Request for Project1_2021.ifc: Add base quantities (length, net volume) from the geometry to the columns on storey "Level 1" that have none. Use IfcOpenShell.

First a look at what the model holds.

```python
import ifcopenshell
import ifcopenshell.util.element
import ifcopenshell.util.unit

model = ifcopenshell.open("Project1_2021.ifc")
print(model.schema)
for unit_type in ("LENGTHUNIT", "AREAUNIT", "VOLUMEUNIT"):
    print(unit_type, ifcopenshell.util.unit.calculate_unit_scale(model, unit_type))
storey = next(s for s in model.by_type("IfcBuildingStorey") if s.Name == "Level 1")
columns = [e for e in ifcopenshell.util.element.get_decomposition(storey) if e.is_a("IfcColumn")]
for e in sorted(columns, key=lambda e: e.id()):
    print(e.id(), e.is_a(), e.Name, list(ifcopenshell.util.element.get_psets(e, qtos_only=True)), sep=" | ")
```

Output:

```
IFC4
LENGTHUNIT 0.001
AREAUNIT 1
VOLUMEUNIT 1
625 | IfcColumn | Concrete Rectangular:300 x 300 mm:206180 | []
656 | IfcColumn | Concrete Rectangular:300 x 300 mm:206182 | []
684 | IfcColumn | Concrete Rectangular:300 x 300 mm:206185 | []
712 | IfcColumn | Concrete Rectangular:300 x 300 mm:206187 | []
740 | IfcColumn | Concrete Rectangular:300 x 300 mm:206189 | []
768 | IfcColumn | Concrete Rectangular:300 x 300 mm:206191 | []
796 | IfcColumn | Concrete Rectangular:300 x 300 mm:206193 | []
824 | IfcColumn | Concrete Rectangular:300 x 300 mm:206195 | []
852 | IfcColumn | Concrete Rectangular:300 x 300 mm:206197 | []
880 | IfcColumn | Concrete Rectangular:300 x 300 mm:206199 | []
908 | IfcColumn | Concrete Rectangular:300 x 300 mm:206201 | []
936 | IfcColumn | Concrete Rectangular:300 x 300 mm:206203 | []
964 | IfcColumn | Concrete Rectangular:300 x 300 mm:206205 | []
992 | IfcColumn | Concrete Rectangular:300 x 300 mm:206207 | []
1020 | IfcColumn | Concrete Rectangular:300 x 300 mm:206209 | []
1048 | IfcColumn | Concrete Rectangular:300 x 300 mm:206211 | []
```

```python
import ifcopenshell
import ifcopenshell.api.pset
import ifcopenshell.geom
import ifcopenshell.util.element
import ifcopenshell.util.shape
import ifcopenshell.util.unit

model = ifcopenshell.open("Project1_2021.ifc")
unit_scale = ifcopenshell.util.unit.calculate_unit_scale(model)
volume_scale = ifcopenshell.util.unit.calculate_unit_scale(model, "VOLUMEUNIT")
settings = ifcopenshell.geom.settings()

storey = next(s for s in model.by_type("IfcBuildingStorey") if s.Name == "Level 1")
columns = [e for e in ifcopenshell.util.element.get_decomposition(storey) if e.is_a("IfcColumn")]

for e in sorted(columns, key=lambda e: e.id()):
    if ifcopenshell.util.element.get_psets(e, qtos_only=True, should_inherit=False):
        continue
    # Geometry comes back in metres, in the element's own axes.
    shape = ifcopenshell.geom.create_shape(settings, e)
    values = {
        "Length": ifcopenshell.util.shape.get_z(shape.geometry) / unit_scale,
        "NetVolume": ifcopenshell.util.shape.get_volume(shape.geometry) / volume_scale,
    }
    qto = ifcopenshell.api.pset.add_qto(model, product=e, name="Qto_ColumnBaseQuantities")
    ifcopenshell.api.pset.edit_qto(model, qto=qto, properties=values)
    print(e.id(), {k: round(v, 3) for k, v in values.items()})

model.write("Project1_2021_rev.ifc")
```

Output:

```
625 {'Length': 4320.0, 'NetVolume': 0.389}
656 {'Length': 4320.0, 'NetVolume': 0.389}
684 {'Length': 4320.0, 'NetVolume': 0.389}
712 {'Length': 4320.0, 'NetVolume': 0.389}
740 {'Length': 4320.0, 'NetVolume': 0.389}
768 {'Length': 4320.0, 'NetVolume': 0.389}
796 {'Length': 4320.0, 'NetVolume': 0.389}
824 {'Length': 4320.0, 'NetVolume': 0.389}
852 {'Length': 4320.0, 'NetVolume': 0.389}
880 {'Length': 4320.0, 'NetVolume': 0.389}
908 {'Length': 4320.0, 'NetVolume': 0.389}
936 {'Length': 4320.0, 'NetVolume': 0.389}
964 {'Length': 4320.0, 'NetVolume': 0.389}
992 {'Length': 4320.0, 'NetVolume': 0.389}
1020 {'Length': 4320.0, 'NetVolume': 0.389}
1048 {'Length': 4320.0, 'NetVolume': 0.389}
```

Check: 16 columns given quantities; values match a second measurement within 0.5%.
